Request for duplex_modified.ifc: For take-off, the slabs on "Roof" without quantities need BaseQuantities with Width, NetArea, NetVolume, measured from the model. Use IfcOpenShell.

First a look at what the model holds.

```python
import ifcopenshell
import ifcopenshell.util.element
import ifcopenshell.util.unit

model = ifcopenshell.open("duplex_modified.ifc")
print(model.schema)
for unit_type in ("LENGTHUNIT", "AREAUNIT", "VOLUMEUNIT"):
    print(unit_type, ifcopenshell.util.unit.calculate_unit_scale(model, unit_type))
storey = next(s for s in model.by_type("IfcBuildingStorey") if s.Name == "Roof")
slabs = [e for e in ifcopenshell.util.element.get_decomposition(storey) if e.is_a("IfcSlab")]
for e in sorted(slabs, key=lambda e: e.id()):
    print(e.id(), e.is_a(), e.Name, list(ifcopenshell.util.element.get_psets(e, qtos_only=True)), sep=" | ")
```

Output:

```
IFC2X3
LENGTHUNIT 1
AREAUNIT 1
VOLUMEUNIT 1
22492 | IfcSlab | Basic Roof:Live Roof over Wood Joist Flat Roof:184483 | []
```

```python
import ifcopenshell
import ifcopenshell.api.pset
import ifcopenshell.geom
import ifcopenshell.util.element
import ifcopenshell.util.shape
import ifcopenshell.util.unit

model = ifcopenshell.open("duplex_modified.ifc")
unit_scale = ifcopenshell.util.unit.calculate_unit_scale(model)
area_scale = ifcopenshell.util.unit.calculate_unit_scale(model, "AREAUNIT")
volume_scale = ifcopenshell.util.unit.calculate_unit_scale(model, "VOLUMEUNIT")
settings = ifcopenshell.geom.settings()

storey = next(s for s in model.by_type("IfcBuildingStorey") if s.Name == "Roof")
slabs = [e for e in ifcopenshell.util.element.get_decomposition(storey) if e.is_a("IfcSlab")]

for e in sorted(slabs, key=lambda e: e.id()):
    if ifcopenshell.util.element.get_psets(e, qtos_only=True, should_inherit=False):
        continue
    # Geometry comes back in metres, in the element's own axes.
    shape = ifcopenshell.geom.create_shape(settings, e)
    values = {
        "Width": ifcopenshell.util.shape.get_z(shape.geometry) / unit_scale,
        "NetArea": ifcopenshell.util.shape.get_footprint_area(shape.geometry) / area_scale,
        "NetVolume": ifcopenshell.util.shape.get_volume(shape.geometry) / volume_scale,
    }
    qto = ifcopenshell.api.pset.add_qto(model, product=e, name="BaseQuantities")
    ifcopenshell.api.pset.edit_qto(model, qto=qto, properties=values)
    print(e.id(), {k: round(v, 3) for k, v in values.items()})

model.write("duplex_modified_rev.ifc")
```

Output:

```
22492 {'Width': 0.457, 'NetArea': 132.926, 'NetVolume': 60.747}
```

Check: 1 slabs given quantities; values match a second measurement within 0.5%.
